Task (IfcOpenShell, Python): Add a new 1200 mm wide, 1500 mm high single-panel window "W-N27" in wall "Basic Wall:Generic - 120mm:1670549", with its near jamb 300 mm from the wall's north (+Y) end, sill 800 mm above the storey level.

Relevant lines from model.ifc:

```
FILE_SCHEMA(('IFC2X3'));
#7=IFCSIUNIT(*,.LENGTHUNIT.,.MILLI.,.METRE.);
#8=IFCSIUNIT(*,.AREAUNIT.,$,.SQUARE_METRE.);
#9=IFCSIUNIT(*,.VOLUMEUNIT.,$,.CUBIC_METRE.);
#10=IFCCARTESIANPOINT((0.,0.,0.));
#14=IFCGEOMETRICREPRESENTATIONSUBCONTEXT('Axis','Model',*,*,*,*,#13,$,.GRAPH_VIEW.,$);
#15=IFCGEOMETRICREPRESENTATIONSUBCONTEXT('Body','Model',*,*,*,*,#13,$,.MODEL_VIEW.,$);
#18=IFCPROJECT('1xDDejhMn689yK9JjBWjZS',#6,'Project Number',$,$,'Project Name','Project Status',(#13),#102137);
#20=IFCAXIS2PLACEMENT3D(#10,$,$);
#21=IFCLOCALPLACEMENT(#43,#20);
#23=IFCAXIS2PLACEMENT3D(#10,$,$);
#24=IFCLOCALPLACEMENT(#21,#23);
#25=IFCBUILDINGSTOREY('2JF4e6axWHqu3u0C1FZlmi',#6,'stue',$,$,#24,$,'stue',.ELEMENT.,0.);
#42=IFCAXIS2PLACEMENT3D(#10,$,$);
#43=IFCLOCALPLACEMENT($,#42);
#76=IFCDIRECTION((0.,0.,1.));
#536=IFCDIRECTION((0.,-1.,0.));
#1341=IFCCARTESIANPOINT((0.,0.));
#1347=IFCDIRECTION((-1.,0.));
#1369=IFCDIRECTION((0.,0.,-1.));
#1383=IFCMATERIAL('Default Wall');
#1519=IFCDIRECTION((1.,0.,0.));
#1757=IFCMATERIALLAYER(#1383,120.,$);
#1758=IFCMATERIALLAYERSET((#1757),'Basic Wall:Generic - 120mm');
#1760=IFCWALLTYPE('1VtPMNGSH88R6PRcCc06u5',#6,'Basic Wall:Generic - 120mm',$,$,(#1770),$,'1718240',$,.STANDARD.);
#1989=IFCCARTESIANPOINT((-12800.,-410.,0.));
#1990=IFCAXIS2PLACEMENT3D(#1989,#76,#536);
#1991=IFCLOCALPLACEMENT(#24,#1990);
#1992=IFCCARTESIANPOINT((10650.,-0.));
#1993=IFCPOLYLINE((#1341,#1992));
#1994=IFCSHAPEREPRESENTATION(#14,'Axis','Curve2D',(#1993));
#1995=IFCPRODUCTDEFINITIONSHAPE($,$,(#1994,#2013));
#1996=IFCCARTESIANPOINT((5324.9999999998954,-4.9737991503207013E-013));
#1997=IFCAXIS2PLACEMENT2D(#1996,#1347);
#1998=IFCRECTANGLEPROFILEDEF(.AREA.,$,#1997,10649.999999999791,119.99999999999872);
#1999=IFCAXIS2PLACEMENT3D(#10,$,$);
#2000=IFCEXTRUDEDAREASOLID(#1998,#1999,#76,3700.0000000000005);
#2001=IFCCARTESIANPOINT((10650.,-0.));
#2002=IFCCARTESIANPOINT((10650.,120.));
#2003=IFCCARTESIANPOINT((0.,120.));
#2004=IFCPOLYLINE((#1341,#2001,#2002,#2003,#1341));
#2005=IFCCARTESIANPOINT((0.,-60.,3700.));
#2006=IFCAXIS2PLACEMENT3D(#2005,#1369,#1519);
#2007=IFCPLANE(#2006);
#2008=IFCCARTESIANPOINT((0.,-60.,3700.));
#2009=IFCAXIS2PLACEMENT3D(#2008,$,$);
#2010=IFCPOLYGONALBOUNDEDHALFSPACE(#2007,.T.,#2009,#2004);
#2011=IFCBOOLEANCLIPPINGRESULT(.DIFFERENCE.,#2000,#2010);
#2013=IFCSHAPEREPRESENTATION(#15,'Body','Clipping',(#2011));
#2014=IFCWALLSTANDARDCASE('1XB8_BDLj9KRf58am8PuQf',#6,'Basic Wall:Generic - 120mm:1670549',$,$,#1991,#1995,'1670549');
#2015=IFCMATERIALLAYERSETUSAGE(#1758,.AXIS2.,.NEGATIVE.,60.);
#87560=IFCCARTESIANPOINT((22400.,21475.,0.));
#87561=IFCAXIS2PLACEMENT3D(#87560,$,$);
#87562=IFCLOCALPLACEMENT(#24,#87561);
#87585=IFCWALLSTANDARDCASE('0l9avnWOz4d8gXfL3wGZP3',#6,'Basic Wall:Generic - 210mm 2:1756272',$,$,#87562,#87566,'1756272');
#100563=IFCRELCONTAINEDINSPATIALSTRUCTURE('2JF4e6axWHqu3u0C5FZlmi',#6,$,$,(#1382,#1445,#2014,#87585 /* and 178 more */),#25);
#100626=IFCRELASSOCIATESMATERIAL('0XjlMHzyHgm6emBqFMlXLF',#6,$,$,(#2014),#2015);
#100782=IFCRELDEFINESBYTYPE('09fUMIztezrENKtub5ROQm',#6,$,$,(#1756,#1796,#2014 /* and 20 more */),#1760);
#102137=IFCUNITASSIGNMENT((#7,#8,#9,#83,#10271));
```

```python
import numpy as np
import ifcopenshell
import ifcopenshell.api.feature
import ifcopenshell.api.geometry
import ifcopenshell.api.root
import ifcopenshell.api.spatial
import ifcopenshell.api.type
import ifcopenshell.geom
import ifcopenshell.util.element
import ifcopenshell.util.placement
import ifcopenshell.util.representation
import ifcopenshell.util.shape
import ifcopenshell.util.unit

model = ifcopenshell.open("model.ifc")
unit_scale = ifcopenshell.util.unit.calculate_unit_scale(model)
settings = ifcopenshell.geom.settings()


def volume(element):
    """Net volume in cubic metres, openings subtracted."""
    shape = ifcopenshell.geom.create_shape(settings, element)
    return ifcopenshell.util.shape.get_volume(shape.geometry)


wall = model.by_guid("1XB8_BDLj9KRf58am8PuQf")
storey = ifcopenshell.util.element.get_container(wall, ifc_class="IfcBuildingStorey")
context = ifcopenshell.util.representation.get_context(model, "Model", "Body", "MODEL_VIEW")
before = volume(wall)

width, height, from_end, sill = 1.2, 1.5, 0.3, 0.8  # metres

# The wall runs along its own X axis, and the end named is its -X end.
wall_shape = ifcopenshell.geom.create_shape(settings, wall)
x, y, z = ifcopenshell.util.shape.get_vertices(wall_shape.geometry).T
start = x.min() + from_end
face, thickness = float(y.min()), float(y.max() - y.min())
wall_matrix = ifcopenshell.util.placement.get_local_placement(wall.ObjectPlacement)
level = ifcopenshell.util.placement.get_local_placement(storey.ObjectPlacement)[2, 3]


def in_wall(x, y):
    """Placement at x, y metres in the wall's axes, at sill height."""
    matrix = wall_matrix.copy()
    matrix[:, 3] = wall_matrix @ np.array([x / unit_scale, y / unit_scale, 0.0, 1.0])
    matrix[2, 3] = level + sill / unit_scale
    return matrix


# Opening: a box that overshoots both wall faces by 50 mm.
opening = ifcopenshell.api.root.create_entity(model, ifc_class="IfcOpeningElement")
box = ifcopenshell.api.geometry.add_wall_representation(
    model, context=context, length=width, height=height, thickness=thickness + 0.1
)
ifcopenshell.api.geometry.assign_representation(model, product=opening, representation=box)
ifcopenshell.api.geometry.edit_object_placement(model, product=opening, matrix=in_wall(start, face - 0.05), is_si=False)
ifcopenshell.api.feature.add_feature(model, feature=opening, element=wall)

window = ifcopenshell.api.root.create_entity(model, ifc_class="IfcWindow", name="W-N27")
window.OverallWidth, window.OverallHeight = width / unit_scale, height / unit_scale
body = ifcopenshell.api.geometry.add_window_representation(
    model,
    context=context,
    overall_width=window.OverallWidth,
    overall_height=window.OverallHeight,
    partition_type="SINGLE_PANEL",
)
ifcopenshell.api.geometry.assign_representation(model, product=window, representation=body)
ifcopenshell.api.spatial.assign_container(model, products=[window], relating_structure=storey)
fills = ifcopenshell.api.feature.add_filling(model, opening=opening, element=window)
fills.OwnerHistory = window.OwnerHistory  # required in IFC2X3

# IFC2X3 keeps the operation on the window style.
style = ifcopenshell.api.root.create_entity(model, ifc_class="IfcWindowStyle", name="W-N27")
style.OperationType, style.ConstructionType = "SINGLE_PANEL", "NOTDEFINED"
style.ParameterTakesPrecedence = style.Sizeable = False
ifcopenshell.api.type.assign_type(model, related_objects=[window], relating_type=style)

# Centre the window in the wall's thickness.
ifcopenshell.api.geometry.edit_object_placement(model, product=window, matrix=in_wall(start, face), is_si=False)
window_shape = ifcopenshell.geom.create_shape(settings, window)
depth = ifcopenshell.util.shape.get_vertices(window_shape.geometry)[:, 1]
offset = face + thickness / 2 - (depth.min() + depth.max()) / 2
ifcopenshell.api.geometry.edit_object_placement(model, product=window, matrix=in_wall(start, offset), is_si=False)

after = volume(wall)

print(f"wall volume {before:.3f} -> {after:.3f} m3")

model.write("model_edited.ifc")
```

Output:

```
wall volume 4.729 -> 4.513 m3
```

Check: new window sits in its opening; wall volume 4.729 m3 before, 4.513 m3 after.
